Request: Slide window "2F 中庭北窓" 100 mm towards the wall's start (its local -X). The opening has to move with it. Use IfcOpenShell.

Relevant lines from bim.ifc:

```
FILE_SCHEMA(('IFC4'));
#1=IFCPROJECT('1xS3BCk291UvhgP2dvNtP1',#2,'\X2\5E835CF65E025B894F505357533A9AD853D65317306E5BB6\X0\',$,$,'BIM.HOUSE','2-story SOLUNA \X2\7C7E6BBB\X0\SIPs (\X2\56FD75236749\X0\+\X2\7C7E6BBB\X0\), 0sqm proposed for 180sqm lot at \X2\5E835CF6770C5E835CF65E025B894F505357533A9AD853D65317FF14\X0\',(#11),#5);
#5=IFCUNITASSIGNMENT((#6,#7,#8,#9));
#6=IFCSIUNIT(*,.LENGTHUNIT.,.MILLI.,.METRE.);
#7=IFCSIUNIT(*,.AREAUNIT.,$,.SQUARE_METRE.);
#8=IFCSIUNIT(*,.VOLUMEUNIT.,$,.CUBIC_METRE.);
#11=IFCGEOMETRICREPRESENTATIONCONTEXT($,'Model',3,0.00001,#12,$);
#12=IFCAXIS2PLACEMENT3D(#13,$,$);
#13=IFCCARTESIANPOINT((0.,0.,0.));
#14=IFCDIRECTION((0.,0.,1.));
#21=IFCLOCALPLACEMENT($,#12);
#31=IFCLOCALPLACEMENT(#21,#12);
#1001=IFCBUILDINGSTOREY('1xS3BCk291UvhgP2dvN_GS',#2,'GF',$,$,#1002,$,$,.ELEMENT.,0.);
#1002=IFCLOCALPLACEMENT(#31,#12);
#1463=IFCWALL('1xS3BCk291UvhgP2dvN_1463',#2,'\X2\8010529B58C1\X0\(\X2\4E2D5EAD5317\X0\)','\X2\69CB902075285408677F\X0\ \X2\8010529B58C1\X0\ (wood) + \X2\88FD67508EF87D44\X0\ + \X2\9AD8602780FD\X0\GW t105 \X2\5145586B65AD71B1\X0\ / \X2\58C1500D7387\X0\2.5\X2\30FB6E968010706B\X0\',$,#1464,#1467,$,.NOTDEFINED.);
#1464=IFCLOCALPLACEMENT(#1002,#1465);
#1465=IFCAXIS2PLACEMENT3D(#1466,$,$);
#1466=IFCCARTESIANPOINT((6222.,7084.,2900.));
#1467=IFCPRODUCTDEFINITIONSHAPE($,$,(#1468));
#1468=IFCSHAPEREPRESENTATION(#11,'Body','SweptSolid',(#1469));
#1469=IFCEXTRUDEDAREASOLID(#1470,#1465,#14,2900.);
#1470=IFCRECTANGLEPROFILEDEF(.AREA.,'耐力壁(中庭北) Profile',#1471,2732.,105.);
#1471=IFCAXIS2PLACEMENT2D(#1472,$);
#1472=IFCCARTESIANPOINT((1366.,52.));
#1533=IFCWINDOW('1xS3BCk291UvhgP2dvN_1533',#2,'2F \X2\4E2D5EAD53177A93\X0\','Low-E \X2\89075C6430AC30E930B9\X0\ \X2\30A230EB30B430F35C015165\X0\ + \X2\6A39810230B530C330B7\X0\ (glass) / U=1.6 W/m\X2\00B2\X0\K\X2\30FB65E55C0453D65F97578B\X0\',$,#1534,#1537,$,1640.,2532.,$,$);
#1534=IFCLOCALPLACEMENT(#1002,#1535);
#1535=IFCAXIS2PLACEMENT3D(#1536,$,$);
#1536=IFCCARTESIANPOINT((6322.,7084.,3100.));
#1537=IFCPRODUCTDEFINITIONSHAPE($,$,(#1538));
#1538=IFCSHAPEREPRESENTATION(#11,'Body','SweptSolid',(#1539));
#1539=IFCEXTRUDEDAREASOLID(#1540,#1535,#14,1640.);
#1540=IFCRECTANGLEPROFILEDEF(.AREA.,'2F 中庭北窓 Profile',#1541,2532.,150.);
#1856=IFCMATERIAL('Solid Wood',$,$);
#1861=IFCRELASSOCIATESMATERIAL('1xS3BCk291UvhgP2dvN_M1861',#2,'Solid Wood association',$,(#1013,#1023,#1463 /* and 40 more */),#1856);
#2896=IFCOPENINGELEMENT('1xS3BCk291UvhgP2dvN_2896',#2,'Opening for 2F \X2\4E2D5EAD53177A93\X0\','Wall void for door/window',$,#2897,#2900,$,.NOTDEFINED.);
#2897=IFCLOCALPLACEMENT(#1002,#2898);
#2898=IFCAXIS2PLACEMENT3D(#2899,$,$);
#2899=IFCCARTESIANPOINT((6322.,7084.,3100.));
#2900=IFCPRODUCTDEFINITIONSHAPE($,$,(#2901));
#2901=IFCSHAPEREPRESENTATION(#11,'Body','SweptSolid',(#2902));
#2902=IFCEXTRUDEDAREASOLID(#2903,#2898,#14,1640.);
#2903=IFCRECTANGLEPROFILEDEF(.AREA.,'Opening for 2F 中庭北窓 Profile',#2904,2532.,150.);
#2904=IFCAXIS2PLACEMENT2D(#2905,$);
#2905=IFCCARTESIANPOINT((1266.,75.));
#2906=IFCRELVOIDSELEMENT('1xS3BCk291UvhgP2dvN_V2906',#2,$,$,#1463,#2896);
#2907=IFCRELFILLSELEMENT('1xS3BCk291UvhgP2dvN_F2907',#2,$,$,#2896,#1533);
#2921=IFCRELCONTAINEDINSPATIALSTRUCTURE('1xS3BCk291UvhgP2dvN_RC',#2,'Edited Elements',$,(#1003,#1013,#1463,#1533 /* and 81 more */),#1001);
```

```python
import ifcopenshell
import ifcopenshell.api.geometry
import ifcopenshell.util.placement

model = ifcopenshell.open("bim.ifc")

window = model.by_guid("1xS3BCk291UvhgP2dvN_1533")
opening = window.FillsVoids[0].RelatingOpeningElement
wall = opening.VoidsElements[0].RelatingBuildingElement

wall_matrix = ifcopenshell.util.placement.get_local_placement(wall.ObjectPlacement)
shift = wall_matrix[:3, 0] * -100.0
before = ifcopenshell.util.placement.get_local_placement(window.ObjectPlacement)[:3, 3].copy()

# The window is not placed relative to its opening, so move both.
for product in (opening, window):
    matrix = ifcopenshell.util.placement.get_local_placement(product.ObjectPlacement)
    matrix[:3, 3] += shift
    ifcopenshell.api.geometry.edit_object_placement(model, product=product, matrix=matrix, is_si=False)

after = ifcopenshell.util.placement.get_local_placement(window.ObjectPlacement)[:3, 3]
print("window moved by", (after - before).round(3) + 0.0)

model.write("bim_edited.ifc")
```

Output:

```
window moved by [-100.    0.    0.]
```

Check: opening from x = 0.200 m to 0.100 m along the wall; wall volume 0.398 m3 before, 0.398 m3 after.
